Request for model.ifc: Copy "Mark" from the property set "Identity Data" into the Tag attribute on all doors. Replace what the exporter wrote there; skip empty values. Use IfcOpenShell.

First a look at what the model holds.

```python
import ifcopenshell
import ifcopenshell.util.element

model = ifcopenshell.open("model.ifc")
print(model.schema)
doors = model.by_type("IfcDoor")
print(len(doors), "doors")
for e in doors[:8]:
    source = ifcopenshell.util.element.get_pset(e, "Identity Data", "Mark")
    target = e.Tag
    print(e.id(), repr(source), repr(target), sep=" | ")
```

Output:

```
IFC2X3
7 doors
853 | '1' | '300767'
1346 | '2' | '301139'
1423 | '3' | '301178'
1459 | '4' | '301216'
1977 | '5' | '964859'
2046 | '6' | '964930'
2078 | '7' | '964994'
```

```python
import ifcopenshell
import ifcopenshell.util.element

model = ifcopenshell.open("model.ifc")

count = 0
for e in model.by_type("IfcDoor"):
    value = ifcopenshell.util.element.get_pset(e, "Identity Data", "Mark")
    current = e.Tag
    if not value or not value.strip() or current == value:
        continue
    e.Tag = value
    count += 1

print(count, "doors updated")

model.write("model_updated.ifc")
```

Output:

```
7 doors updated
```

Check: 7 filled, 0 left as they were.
